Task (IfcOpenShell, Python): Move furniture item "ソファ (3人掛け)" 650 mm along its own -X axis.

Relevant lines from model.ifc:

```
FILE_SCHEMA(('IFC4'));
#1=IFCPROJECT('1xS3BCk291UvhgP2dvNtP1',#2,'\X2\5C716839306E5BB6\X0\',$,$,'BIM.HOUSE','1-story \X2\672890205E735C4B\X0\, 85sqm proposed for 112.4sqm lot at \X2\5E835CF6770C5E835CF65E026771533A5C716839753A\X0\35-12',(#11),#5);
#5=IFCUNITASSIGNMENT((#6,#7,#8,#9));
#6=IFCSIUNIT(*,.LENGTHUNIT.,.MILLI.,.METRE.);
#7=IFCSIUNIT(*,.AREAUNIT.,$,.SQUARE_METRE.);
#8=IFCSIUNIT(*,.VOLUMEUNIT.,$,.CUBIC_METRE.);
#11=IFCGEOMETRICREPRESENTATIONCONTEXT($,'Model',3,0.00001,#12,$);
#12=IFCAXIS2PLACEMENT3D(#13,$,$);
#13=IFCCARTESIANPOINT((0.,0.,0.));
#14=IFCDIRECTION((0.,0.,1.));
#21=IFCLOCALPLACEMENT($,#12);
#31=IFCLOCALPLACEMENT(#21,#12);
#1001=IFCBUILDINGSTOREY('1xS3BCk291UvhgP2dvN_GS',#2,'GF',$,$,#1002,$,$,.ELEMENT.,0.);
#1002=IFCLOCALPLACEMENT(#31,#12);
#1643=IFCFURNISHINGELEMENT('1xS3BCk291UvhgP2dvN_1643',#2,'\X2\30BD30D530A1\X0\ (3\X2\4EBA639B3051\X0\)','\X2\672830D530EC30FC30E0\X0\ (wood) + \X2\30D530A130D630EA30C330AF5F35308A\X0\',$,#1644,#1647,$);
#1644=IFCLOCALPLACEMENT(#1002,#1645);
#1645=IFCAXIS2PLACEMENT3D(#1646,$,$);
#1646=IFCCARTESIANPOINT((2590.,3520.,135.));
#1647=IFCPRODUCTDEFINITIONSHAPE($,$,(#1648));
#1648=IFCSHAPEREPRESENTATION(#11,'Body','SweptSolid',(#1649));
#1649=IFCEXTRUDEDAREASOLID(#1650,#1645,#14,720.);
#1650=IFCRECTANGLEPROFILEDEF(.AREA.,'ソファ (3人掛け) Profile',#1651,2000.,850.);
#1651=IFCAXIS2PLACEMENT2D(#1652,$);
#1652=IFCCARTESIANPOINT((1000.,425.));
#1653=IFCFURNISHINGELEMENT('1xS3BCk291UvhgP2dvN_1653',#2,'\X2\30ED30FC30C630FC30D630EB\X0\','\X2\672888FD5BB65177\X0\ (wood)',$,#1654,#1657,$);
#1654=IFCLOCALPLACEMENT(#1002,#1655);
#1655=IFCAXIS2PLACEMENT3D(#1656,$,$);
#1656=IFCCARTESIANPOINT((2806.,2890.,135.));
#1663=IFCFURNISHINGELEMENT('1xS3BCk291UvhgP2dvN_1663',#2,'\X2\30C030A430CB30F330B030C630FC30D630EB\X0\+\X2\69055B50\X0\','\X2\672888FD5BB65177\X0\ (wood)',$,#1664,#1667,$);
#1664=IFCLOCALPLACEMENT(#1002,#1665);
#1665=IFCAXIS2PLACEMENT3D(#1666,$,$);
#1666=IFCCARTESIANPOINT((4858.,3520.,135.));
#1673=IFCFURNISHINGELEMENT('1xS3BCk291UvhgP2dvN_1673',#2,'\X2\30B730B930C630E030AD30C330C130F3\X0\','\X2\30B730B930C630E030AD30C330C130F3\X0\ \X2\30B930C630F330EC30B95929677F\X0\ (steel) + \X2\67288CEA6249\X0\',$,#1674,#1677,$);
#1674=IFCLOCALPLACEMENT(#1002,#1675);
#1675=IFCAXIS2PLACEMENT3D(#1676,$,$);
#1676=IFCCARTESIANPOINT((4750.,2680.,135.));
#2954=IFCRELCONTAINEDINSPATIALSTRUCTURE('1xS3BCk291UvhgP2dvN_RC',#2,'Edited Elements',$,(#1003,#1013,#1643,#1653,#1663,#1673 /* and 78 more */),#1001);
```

```python
import ifcopenshell
import ifcopenshell.api.geometry
import ifcopenshell.util.placement
import ifcopenshell.util.unit

model = ifcopenshell.open("model.ifc")
unit_scale = ifcopenshell.util.unit.calculate_unit_scale(model)

item = model.by_guid("1xS3BCk291UvhgP2dvN_1643")
matrix = ifcopenshell.util.placement.get_local_placement(item.ObjectPlacement)
matrix[:3, 3] -= matrix[:3, 0] * 0.65 / unit_scale
ifcopenshell.api.geometry.edit_object_placement(model, product=item, matrix=matrix, is_si=False)

print(ifcopenshell.util.placement.get_local_placement(item.ObjectPlacement).round(3) + 0.0)

model.write("model_rev.ifc")
```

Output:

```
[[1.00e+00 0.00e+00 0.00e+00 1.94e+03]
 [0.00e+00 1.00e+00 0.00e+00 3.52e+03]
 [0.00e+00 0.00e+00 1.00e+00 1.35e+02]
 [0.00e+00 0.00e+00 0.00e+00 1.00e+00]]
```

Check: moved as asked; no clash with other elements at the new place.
